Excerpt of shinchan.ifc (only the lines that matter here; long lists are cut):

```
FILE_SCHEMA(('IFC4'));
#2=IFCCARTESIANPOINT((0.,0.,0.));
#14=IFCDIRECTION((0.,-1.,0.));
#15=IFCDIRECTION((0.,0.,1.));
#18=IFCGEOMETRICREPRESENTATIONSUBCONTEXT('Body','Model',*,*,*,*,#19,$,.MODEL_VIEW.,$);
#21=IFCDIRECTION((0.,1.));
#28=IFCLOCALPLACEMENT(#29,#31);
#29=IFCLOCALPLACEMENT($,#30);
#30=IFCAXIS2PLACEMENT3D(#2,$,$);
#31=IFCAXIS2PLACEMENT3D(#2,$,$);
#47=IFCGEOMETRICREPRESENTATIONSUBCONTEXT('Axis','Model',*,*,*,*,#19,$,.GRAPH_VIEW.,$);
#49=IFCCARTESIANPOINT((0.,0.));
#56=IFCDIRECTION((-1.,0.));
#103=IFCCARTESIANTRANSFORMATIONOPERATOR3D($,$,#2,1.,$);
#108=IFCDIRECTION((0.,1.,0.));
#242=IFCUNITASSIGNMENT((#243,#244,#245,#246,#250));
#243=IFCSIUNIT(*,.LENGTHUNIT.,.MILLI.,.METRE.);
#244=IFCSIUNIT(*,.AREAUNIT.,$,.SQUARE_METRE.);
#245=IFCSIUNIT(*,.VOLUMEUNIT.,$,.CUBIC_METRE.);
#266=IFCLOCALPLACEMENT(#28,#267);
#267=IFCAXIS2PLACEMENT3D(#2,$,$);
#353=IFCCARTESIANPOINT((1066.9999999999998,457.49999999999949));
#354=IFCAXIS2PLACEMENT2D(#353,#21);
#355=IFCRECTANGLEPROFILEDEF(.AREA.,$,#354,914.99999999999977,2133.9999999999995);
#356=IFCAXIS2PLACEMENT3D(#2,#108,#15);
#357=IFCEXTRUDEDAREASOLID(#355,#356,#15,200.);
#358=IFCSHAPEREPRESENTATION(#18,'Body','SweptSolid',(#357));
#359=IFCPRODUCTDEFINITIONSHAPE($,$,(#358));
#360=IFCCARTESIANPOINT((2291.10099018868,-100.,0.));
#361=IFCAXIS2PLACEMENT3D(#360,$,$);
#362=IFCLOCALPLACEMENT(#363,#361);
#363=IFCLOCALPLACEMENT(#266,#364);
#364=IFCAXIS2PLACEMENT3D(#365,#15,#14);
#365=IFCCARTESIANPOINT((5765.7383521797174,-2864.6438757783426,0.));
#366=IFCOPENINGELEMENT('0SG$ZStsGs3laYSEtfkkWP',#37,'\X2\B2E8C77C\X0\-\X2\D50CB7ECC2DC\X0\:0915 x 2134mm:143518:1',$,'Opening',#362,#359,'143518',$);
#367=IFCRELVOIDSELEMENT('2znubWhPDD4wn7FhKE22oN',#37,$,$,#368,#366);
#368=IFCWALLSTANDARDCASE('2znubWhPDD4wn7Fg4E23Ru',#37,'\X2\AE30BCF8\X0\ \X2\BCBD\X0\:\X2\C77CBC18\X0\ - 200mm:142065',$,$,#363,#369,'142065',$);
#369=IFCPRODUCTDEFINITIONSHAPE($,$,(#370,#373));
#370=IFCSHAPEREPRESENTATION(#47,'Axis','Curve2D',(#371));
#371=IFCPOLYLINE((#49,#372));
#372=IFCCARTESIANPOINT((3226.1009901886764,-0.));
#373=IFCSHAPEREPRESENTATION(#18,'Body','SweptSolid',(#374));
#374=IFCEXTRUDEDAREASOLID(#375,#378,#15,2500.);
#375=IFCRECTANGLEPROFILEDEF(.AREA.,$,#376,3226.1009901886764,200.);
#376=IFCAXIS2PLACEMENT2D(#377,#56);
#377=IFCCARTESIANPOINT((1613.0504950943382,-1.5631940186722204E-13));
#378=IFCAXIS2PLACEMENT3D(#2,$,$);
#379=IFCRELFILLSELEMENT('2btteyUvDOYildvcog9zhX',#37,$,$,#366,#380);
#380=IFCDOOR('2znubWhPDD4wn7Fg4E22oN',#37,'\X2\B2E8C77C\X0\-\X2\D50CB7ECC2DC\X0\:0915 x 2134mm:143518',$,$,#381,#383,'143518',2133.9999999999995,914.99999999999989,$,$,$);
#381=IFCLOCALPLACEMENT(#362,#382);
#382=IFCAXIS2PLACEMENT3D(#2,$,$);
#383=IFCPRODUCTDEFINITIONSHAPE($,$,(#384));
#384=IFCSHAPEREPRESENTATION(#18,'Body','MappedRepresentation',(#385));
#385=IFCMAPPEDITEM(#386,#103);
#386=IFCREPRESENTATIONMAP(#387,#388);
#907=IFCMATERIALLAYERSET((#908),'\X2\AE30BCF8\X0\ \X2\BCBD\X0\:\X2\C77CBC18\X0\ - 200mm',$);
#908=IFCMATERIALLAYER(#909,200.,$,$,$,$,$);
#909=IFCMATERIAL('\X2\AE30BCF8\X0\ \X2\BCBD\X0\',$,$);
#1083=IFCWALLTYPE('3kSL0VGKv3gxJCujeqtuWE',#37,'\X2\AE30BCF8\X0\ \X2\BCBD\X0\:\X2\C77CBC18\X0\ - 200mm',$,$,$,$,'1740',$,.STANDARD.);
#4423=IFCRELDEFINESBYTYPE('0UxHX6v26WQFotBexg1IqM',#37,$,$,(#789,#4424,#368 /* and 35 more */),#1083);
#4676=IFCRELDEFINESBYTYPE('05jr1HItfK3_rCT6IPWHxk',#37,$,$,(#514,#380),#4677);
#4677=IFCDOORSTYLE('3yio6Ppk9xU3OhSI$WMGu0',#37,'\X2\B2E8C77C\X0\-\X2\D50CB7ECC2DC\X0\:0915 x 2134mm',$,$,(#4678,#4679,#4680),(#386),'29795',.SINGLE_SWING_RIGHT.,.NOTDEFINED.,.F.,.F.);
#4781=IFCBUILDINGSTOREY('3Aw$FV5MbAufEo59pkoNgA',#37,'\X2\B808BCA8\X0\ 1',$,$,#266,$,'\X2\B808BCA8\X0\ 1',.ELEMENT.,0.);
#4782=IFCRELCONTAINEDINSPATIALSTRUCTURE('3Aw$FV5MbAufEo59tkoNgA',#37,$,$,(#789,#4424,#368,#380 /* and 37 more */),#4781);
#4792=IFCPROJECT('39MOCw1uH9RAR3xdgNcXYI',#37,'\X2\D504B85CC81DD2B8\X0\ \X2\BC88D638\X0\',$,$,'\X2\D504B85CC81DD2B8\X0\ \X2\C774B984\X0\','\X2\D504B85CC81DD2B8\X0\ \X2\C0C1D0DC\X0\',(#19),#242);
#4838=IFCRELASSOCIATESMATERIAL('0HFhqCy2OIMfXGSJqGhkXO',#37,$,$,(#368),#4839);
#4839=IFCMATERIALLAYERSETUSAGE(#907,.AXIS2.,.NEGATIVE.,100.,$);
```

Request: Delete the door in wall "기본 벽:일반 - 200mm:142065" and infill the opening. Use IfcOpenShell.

```python
import ifcopenshell
import ifcopenshell.api.feature
import ifcopenshell.api.root
import ifcopenshell.geom
import ifcopenshell.util.shape

model = ifcopenshell.open("shinchan.ifc")
settings = ifcopenshell.geom.settings()


def volume(element):
    """Net volume in cubic metres, openings subtracted."""
    shape = ifcopenshell.geom.create_shape(settings, element)
    return ifcopenshell.util.shape.get_volume(shape.geometry)


door = model.by_guid("2znubWhPDD4wn7Fg4E22oN")
opening = door.FillsVoids[0].RelatingOpeningElement
wall = opening.VoidsElements[0].RelatingBuildingElement
before = volume(wall)

ifcopenshell.api.root.remove_product(model, product=door)
ifcopenshell.api.feature.remove_feature(model, feature=opening)

after = volume(wall)

print(f"wall volume {before:.3f} -> {after:.3f} m3")

model.write("shinchan-out.ifc")
```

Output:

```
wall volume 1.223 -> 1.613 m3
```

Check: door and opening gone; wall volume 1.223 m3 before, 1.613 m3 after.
